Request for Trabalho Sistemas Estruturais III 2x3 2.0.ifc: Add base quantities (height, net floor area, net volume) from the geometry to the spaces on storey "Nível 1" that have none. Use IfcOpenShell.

First a look at what the model holds.

```python
import ifcopenshell
import ifcopenshell.util.element
import ifcopenshell.util.unit

model = ifcopenshell.open("Trabalho Sistemas Estruturais III 2x3 2.0.ifc")
print(model.schema)
for unit_type in ("LENGTHUNIT", "AREAUNIT", "VOLUMEUNIT"):
    print(unit_type, ifcopenshell.util.unit.calculate_unit_scale(model, unit_type))
storey = next(s for s in model.by_type("IfcBuildingStorey") if s.Name == "Nível 1")
spaces = [e for e in ifcopenshell.util.element.get_decomposition(storey) if e.is_a("IfcSpace")]
for e in sorted(spaces, key=lambda e: e.id()):
    print(e.id(), e.is_a(), e.Name, list(ifcopenshell.util.element.get_psets(e, qtos_only=True)), sep=" | ")
```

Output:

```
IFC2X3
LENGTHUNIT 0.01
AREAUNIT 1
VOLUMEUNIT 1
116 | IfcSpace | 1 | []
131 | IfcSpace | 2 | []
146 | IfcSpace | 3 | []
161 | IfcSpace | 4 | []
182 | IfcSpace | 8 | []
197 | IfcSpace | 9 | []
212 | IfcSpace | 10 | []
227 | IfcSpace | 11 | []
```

```python
import ifcopenshell
import ifcopenshell.api.pset
import ifcopenshell.geom
import ifcopenshell.util.element
import ifcopenshell.util.shape
import ifcopenshell.util.unit

model = ifcopenshell.open("Trabalho Sistemas Estruturais III 2x3 2.0.ifc")
unit_scale = ifcopenshell.util.unit.calculate_unit_scale(model)
area_scale = ifcopenshell.util.unit.calculate_unit_scale(model, "AREAUNIT")
volume_scale = ifcopenshell.util.unit.calculate_unit_scale(model, "VOLUMEUNIT")
settings = ifcopenshell.geom.settings()

storey = next(s for s in model.by_type("IfcBuildingStorey") if s.Name == "Nível 1")
spaces = [e for e in ifcopenshell.util.element.get_decomposition(storey) if e.is_a("IfcSpace")]

for e in sorted(spaces, key=lambda e: e.id()):
    if ifcopenshell.util.element.get_psets(e, qtos_only=True, should_inherit=False):
        continue
    # Geometry comes back in metres, in the element's own axes.
    shape = ifcopenshell.geom.create_shape(settings, e)
    values = {
        "Height": ifcopenshell.util.shape.get_z(shape.geometry) / unit_scale,
        "NetFloorArea": ifcopenshell.util.shape.get_footprint_area(shape.geometry) / area_scale,
        "NetVolume": ifcopenshell.util.shape.get_volume(shape.geometry) / volume_scale,
    }
    qto = ifcopenshell.api.pset.add_qto(model, product=e, name="BaseQuantities")
    ifcopenshell.api.pset.edit_qto(model, qto=qto, properties=values)
    print(e.id(), {k: round(v, 3) for k, v in values.items()})

model.write("Trabalho Sistemas Estruturais III 2x3 2.0_v2.ifc")
```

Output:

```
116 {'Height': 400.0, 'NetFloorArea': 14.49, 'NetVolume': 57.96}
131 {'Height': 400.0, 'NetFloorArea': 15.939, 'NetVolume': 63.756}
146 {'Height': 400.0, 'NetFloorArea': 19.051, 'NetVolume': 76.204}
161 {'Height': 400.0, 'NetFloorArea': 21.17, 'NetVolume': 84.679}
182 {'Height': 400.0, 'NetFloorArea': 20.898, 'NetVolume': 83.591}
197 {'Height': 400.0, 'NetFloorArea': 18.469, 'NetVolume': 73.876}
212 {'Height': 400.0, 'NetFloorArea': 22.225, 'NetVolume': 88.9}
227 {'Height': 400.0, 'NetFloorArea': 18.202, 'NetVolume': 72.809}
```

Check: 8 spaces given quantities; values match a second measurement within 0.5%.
